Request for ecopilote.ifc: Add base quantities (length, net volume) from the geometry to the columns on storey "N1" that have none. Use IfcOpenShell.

First a look at what the model holds.

```python
import ifcopenshell
import ifcopenshell.util.element
import ifcopenshell.util.unit

model = ifcopenshell.open("ecopilote.ifc")
print(model.schema)
for unit_type in ("LENGTHUNIT", "AREAUNIT", "VOLUMEUNIT"):
    print(unit_type, ifcopenshell.util.unit.calculate_unit_scale(model, unit_type))
storey = next(s for s in model.by_type("IfcBuildingStorey") if s.Name == "N1")
columns = [e for e in ifcopenshell.util.element.get_decomposition(storey) if e.is_a("IfcColumn")]
for e in sorted(columns, key=lambda e: e.id()):
    print(e.id(), e.is_a(), e.Name, list(ifcopenshell.util.element.get_psets(e, qtos_only=True)), sep=" | ")
```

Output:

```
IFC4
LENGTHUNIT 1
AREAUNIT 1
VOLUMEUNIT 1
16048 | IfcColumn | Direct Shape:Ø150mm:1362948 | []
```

```python
import ifcopenshell
import ifcopenshell.api.pset
import ifcopenshell.geom
import ifcopenshell.util.element
import ifcopenshell.util.shape
import ifcopenshell.util.unit

model = ifcopenshell.open("ecopilote.ifc")
unit_scale = ifcopenshell.util.unit.calculate_unit_scale(model)
volume_scale = ifcopenshell.util.unit.calculate_unit_scale(model, "VOLUMEUNIT")
settings = ifcopenshell.geom.settings()

storey = next(s for s in model.by_type("IfcBuildingStorey") if s.Name == "N1")
columns = [e for e in ifcopenshell.util.element.get_decomposition(storey) if e.is_a("IfcColumn")]

for e in sorted(columns, key=lambda e: e.id()):
    if ifcopenshell.util.element.get_psets(e, qtos_only=True, should_inherit=False):
        continue
    # Geometry comes back in metres, in the element's own axes.
    shape = ifcopenshell.geom.create_shape(settings, e)
    values = {
        "Length": ifcopenshell.util.shape.get_z(shape.geometry) / unit_scale,
        "NetVolume": ifcopenshell.util.shape.get_volume(shape.geometry) / volume_scale,
    }
    qto = ifcopenshell.api.pset.add_qto(model, product=e, name="Qto_ColumnBaseQuantities")
    ifcopenshell.api.pset.edit_qto(model, qto=qto, properties=values)
    print(e.id(), {k: round(v, 3) for k, v in values.items()})

model.write("ecopilote_edited.ifc")
```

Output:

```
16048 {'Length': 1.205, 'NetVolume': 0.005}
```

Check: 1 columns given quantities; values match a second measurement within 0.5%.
